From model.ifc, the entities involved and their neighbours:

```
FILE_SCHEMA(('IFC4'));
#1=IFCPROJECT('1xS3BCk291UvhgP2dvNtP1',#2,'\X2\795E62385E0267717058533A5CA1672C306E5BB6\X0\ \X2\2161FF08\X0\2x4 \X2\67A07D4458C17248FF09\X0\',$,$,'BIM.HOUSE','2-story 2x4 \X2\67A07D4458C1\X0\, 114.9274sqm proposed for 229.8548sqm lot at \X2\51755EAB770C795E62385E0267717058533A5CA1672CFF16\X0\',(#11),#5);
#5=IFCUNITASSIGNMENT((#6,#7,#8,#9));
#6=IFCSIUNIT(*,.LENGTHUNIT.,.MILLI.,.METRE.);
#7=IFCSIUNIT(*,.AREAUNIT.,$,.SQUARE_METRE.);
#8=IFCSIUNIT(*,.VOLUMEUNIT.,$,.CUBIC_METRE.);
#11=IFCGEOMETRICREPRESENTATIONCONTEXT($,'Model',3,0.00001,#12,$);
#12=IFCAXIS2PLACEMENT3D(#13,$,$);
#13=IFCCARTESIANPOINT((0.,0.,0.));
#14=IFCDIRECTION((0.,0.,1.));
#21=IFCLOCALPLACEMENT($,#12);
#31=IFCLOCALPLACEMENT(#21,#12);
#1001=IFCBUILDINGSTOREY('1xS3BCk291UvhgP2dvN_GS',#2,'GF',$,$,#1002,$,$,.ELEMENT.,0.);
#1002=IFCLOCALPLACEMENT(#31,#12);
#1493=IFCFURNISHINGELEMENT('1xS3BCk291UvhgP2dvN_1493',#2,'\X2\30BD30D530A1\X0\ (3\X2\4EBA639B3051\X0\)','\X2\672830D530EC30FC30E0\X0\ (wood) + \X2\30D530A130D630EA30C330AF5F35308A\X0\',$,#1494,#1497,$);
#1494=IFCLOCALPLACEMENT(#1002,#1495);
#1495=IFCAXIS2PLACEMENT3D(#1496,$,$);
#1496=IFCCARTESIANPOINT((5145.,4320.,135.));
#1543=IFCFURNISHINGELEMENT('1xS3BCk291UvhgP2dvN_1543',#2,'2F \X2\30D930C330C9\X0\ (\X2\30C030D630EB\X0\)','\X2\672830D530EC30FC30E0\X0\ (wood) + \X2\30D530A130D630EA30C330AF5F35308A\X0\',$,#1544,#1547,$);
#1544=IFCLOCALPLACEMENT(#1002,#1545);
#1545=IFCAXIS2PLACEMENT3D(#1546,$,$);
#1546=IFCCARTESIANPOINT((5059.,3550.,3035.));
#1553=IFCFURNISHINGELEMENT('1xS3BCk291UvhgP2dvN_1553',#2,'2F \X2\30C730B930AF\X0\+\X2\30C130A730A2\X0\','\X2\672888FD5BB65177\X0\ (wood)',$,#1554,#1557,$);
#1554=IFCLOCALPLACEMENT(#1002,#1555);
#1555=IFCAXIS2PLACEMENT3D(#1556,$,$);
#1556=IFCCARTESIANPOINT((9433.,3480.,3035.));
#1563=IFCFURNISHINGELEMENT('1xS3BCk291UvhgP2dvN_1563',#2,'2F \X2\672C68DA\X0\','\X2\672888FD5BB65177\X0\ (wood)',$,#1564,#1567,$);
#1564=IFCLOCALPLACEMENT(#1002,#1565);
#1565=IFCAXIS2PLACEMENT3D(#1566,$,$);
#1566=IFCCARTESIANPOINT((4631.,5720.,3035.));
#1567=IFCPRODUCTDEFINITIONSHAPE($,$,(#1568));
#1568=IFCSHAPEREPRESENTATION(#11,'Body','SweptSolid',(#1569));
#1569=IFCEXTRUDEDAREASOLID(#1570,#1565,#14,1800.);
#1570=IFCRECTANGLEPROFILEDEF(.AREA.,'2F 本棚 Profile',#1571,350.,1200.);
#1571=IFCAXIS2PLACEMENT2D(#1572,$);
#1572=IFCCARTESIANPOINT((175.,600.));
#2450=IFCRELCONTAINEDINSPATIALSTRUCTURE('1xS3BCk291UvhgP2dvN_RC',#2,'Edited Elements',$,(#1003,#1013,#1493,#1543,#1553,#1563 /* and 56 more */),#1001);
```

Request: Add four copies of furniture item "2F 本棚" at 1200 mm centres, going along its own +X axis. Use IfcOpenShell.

```python
import ifcopenshell
import ifcopenshell.api.geometry
import ifcopenshell.api.root
import ifcopenshell.util.element
import ifcopenshell.util.placement
import ifcopenshell.util.unit

model = ifcopenshell.open("model.ifc")
unit_scale = ifcopenshell.util.unit.calculate_unit_scale(model)


def reuse_history(source, copy):
    """copy_class also copies each property set's owner history, people and application; keep the originals."""
    for rel in copy.IsDefinedBy:
        if rel.is_a("IfcRelDefinesByProperties") and (history := rel.RelatingPropertyDefinition.OwnerHistory):
            rel.RelatingPropertyDefinition.OwnerHistory = source.OwnerHistory
            ifcopenshell.util.element.remove_deep2(model, history)


source = model.by_guid("1xS3BCk291UvhgP2dvN_1563")
base = ifcopenshell.util.placement.get_local_placement(source.ObjectPlacement)
step = base[:3, 0] * 1.2 / unit_scale

for i in range(1, 5):
    copy = ifcopenshell.api.root.copy_class(model, product=source)
    copy.Representation = ifcopenshell.util.element.copy_deep(
        model, source.Representation, exclude=["IfcGeometricRepresentationContext", "IfcRepresentationMap"]
    )
    reuse_history(source, copy)
    matrix = base.copy()
    matrix[:3, 3] += i * step
    print("added at", matrix[:3, 3].round(3) + 0.0)
    ifcopenshell.api.geometry.edit_object_placement(model, product=copy, matrix=matrix, is_si=False)

model.write("model_rev.ifc")
```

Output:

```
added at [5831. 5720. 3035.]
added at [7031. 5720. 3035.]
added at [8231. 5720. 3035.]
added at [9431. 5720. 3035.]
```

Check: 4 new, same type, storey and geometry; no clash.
